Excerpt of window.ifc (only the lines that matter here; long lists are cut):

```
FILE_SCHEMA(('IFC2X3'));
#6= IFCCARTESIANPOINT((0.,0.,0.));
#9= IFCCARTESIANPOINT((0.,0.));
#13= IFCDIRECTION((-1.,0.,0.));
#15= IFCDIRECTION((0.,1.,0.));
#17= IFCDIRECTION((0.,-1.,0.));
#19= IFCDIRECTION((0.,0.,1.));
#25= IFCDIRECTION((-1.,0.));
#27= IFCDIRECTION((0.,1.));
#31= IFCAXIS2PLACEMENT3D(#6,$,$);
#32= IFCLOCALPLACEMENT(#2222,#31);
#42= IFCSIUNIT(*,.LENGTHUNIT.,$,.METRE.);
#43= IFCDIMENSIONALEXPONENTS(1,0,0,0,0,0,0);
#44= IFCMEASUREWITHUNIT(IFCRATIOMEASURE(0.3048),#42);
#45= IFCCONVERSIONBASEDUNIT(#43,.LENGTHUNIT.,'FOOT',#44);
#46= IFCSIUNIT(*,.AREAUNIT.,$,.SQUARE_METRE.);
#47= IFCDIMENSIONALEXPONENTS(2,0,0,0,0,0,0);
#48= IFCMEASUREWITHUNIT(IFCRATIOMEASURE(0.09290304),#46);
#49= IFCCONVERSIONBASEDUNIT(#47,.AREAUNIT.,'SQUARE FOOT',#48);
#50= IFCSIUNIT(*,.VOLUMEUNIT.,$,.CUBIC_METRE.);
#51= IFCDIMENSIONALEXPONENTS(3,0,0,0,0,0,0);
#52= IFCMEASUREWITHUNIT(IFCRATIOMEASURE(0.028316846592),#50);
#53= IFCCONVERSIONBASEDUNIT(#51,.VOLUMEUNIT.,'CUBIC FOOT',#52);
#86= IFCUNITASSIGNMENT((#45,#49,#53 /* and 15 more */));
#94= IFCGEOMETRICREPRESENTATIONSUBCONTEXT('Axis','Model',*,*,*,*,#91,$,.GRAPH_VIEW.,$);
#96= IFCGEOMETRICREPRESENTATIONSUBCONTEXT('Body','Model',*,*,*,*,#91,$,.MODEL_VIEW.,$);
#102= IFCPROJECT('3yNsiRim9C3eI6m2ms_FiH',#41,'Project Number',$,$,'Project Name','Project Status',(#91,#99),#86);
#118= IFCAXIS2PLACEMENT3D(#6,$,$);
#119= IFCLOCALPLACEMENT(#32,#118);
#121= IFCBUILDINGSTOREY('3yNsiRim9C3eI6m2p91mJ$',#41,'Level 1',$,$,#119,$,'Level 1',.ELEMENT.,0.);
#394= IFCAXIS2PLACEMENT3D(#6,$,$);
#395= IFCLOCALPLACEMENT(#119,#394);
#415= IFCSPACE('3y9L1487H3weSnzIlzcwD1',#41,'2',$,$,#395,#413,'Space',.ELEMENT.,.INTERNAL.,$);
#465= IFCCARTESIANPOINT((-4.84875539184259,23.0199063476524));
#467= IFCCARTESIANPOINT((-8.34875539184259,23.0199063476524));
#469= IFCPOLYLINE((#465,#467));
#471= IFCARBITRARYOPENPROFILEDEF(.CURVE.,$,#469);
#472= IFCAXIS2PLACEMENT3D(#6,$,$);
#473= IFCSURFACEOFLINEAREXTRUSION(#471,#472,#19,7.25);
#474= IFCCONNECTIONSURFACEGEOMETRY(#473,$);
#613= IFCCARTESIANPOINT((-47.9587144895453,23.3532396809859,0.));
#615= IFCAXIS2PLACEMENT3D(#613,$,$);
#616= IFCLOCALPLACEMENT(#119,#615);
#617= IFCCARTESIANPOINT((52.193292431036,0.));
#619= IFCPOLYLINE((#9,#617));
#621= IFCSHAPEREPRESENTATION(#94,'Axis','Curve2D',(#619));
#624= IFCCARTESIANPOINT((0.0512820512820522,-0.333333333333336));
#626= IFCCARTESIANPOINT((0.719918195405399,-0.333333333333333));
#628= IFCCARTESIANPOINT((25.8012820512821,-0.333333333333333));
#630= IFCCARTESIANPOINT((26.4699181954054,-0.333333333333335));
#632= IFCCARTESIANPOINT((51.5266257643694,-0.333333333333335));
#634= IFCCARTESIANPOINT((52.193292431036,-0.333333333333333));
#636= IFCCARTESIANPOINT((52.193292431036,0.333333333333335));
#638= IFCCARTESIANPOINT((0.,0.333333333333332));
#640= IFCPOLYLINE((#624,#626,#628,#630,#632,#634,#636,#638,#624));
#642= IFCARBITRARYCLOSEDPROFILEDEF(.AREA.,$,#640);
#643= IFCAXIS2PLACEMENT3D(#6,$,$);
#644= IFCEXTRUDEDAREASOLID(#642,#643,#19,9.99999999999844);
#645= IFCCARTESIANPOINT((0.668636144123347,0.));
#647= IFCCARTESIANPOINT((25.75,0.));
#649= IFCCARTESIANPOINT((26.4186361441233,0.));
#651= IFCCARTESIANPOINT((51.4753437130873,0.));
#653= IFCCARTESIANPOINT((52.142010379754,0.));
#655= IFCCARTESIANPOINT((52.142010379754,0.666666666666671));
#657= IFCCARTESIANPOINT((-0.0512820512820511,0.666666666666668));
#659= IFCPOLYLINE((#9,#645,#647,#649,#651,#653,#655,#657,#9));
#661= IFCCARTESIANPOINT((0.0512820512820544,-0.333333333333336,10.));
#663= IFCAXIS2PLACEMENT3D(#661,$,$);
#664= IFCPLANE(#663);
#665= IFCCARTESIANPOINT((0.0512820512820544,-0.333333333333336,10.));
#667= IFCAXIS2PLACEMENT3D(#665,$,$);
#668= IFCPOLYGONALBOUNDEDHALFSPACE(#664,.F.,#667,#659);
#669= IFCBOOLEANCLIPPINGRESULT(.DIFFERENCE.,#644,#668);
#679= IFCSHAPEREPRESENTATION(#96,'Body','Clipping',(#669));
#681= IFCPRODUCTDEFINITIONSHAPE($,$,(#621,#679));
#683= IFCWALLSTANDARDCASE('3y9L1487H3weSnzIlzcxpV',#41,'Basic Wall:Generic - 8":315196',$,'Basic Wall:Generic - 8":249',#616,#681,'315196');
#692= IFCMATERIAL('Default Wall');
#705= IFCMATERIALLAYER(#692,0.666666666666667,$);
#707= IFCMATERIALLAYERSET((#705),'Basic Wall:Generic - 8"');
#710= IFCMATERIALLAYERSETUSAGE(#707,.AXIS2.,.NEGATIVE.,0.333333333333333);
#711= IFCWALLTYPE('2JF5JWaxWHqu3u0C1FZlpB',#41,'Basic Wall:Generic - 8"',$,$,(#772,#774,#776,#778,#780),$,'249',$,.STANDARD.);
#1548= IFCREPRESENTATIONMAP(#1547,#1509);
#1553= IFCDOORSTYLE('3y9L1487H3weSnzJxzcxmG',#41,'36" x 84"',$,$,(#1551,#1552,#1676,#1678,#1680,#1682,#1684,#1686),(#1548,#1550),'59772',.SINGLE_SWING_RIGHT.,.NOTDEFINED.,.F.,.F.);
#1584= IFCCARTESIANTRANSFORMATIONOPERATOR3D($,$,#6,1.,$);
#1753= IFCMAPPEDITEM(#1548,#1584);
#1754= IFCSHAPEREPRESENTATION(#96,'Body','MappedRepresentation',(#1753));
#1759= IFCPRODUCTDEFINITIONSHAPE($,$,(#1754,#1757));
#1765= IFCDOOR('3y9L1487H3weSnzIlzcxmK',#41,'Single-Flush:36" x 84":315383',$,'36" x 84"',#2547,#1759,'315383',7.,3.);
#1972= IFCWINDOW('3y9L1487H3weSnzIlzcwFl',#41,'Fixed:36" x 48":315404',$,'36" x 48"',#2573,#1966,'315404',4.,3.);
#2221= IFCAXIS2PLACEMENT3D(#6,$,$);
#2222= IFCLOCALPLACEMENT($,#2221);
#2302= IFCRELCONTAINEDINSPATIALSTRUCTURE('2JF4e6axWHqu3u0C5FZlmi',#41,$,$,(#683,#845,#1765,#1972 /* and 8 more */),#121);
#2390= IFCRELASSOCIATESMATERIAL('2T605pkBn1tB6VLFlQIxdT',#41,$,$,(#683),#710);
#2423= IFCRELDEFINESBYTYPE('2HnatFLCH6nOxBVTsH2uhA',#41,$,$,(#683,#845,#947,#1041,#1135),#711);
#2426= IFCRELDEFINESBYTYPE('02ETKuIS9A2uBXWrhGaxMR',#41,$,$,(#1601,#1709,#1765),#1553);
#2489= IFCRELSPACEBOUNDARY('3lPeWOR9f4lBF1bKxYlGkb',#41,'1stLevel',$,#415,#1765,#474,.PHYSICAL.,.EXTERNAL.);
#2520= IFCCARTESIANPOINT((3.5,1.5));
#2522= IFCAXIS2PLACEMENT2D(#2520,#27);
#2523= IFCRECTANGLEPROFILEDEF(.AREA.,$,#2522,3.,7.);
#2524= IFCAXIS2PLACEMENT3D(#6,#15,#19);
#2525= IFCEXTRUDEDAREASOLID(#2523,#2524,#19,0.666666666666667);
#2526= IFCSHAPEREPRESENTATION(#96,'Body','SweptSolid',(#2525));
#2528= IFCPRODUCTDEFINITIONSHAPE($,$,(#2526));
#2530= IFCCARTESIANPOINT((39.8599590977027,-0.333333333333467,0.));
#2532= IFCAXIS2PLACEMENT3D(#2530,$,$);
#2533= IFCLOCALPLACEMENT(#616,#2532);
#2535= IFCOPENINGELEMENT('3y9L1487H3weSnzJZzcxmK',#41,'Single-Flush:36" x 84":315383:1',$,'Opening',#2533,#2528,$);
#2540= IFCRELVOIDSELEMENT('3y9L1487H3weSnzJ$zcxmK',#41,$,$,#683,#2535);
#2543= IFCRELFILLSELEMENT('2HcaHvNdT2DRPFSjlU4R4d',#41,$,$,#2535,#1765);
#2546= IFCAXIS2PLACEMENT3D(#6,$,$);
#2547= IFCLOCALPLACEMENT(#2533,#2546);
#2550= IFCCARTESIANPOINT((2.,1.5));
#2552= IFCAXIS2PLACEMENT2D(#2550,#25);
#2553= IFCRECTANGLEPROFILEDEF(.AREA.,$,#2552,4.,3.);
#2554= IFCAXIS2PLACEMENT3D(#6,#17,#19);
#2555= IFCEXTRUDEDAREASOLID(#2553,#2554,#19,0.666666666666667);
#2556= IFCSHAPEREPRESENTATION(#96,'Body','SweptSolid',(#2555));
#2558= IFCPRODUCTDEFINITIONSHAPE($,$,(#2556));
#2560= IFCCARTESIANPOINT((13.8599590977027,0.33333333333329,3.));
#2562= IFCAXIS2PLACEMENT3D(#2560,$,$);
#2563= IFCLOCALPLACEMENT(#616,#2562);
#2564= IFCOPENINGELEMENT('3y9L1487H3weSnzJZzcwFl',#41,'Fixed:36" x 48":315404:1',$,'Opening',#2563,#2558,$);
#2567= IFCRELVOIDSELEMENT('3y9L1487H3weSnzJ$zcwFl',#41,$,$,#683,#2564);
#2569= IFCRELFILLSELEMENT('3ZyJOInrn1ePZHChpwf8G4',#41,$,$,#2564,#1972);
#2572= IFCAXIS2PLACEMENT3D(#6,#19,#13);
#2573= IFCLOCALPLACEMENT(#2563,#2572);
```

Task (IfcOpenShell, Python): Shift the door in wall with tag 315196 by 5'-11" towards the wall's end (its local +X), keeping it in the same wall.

```python
import numpy as np
import ifcopenshell
import ifcopenshell.api.geometry
import ifcopenshell.util.placement
import ifcopenshell.util.unit

model = ifcopenshell.open("window.ifc")
unit_scale = ifcopenshell.util.unit.calculate_unit_scale(model)

door = model.by_guid("3y9L1487H3weSnzIlzcxmK")
opening = door.FillsVoids[0].RelatingOpeningElement
wall = opening.VoidsElements[0].RelatingBuildingElement

wall_matrix = ifcopenshell.util.placement.get_local_placement(wall.ObjectPlacement)
shift = wall_matrix[:3, 0] * 71 * 0.0254 / unit_scale
before = ifcopenshell.util.placement.get_local_placement(door.ObjectPlacement)[:3, 3].copy()

# The door is placed relative to its opening, so it follows when the opening moves.
matrix = ifcopenshell.util.placement.get_local_placement(opening.ObjectPlacement)
matrix[:3, 3] += shift
ifcopenshell.api.geometry.edit_object_placement(
    model, product=opening, matrix=matrix, is_si=False, should_transform_children=True
)

# Space boundary surfaces are stored in each space's coordinates; move them too.
for rel in door.ProvidesBoundaries:
    if not rel.ConnectionGeometry:
        continue
    surface = rel.ConnectionGeometry.SurfaceOnRelatingElement
    space_matrix = ifcopenshell.util.placement.get_local_placement(rel.RelatingSpace.ObjectPlacement)
    point = np.array(surface.Position.Location.Coordinates) + space_matrix[:3, :3].T @ shift
    surface.Position = model.createIfcAxis2Placement3D(
        model.createIfcCartesianPoint(point.tolist()), surface.Position.Axis, surface.Position.RefDirection
    )

after = ifcopenshell.util.placement.get_local_placement(door.ObjectPlacement)[:3, 3]
print("door moved by", (after - before).round(3) + 0.0)

model.write("window-out.ifc")
```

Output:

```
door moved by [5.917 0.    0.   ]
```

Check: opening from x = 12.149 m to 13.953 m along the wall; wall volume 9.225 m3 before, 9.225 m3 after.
